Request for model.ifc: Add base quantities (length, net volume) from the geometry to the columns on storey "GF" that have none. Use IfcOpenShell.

First a look at what the model holds.

```python
import ifcopenshell
import ifcopenshell.util.element
import ifcopenshell.util.unit

model = ifcopenshell.open("model.ifc")
print(model.schema)
for unit_type in ("LENGTHUNIT", "AREAUNIT", "VOLUMEUNIT"):
    print(unit_type, ifcopenshell.util.unit.calculate_unit_scale(model, unit_type))
storey = next(s for s in model.by_type("IfcBuildingStorey") if s.Name == "GF")
columns = [e for e in ifcopenshell.util.element.get_decomposition(storey) if e.is_a("IfcColumn")]
for e in sorted(columns, key=lambda e: e.id()):
    print(e.id(), e.is_a(), e.Name, list(ifcopenshell.util.element.get_psets(e, qtos_only=True)), sep=" | ")
```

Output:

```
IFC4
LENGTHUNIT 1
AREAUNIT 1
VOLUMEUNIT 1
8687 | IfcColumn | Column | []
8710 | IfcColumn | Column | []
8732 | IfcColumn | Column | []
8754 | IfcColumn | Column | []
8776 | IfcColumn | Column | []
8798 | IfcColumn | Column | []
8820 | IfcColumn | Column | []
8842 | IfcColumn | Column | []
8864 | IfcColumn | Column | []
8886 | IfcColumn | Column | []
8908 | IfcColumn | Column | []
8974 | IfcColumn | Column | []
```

```python
import ifcopenshell
import ifcopenshell.api.pset
import ifcopenshell.geom
import ifcopenshell.util.element
import ifcopenshell.util.shape
import ifcopenshell.util.unit

model = ifcopenshell.open("model.ifc")
unit_scale = ifcopenshell.util.unit.calculate_unit_scale(model)
volume_scale = ifcopenshell.util.unit.calculate_unit_scale(model, "VOLUMEUNIT")
settings = ifcopenshell.geom.settings()

storey = next(s for s in model.by_type("IfcBuildingStorey") if s.Name == "GF")
columns = [e for e in ifcopenshell.util.element.get_decomposition(storey) if e.is_a("IfcColumn")]

for e in sorted(columns, key=lambda e: e.id()):
    if ifcopenshell.util.element.get_psets(e, qtos_only=True, should_inherit=False):
        continue
    # Geometry comes back in metres, in the element's own axes.
    shape = ifcopenshell.geom.create_shape(settings, e)
    values = {
        "Length": ifcopenshell.util.shape.get_z(shape.geometry) / unit_scale,
        "NetVolume": ifcopenshell.util.shape.get_volume(shape.geometry) / volume_scale,
    }
    qto = ifcopenshell.api.pset.add_qto(model, product=e, name="Qto_ColumnBaseQuantities")
    ifcopenshell.api.pset.edit_qto(model, qto=qto, properties=values)
    print(e.id(), {k: round(v, 3) for k, v in values.items()})

model.write("model_updated.ifc")
```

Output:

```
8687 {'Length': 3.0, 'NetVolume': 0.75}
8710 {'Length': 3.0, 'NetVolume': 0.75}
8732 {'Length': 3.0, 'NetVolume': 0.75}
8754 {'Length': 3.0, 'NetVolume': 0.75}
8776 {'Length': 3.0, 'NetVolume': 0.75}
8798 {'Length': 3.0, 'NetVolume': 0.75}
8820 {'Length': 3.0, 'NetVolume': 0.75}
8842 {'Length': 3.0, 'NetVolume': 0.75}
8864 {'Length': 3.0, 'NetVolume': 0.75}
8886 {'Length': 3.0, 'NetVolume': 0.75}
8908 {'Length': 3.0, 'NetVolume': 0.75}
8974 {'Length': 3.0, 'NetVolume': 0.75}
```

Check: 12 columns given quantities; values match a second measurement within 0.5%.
